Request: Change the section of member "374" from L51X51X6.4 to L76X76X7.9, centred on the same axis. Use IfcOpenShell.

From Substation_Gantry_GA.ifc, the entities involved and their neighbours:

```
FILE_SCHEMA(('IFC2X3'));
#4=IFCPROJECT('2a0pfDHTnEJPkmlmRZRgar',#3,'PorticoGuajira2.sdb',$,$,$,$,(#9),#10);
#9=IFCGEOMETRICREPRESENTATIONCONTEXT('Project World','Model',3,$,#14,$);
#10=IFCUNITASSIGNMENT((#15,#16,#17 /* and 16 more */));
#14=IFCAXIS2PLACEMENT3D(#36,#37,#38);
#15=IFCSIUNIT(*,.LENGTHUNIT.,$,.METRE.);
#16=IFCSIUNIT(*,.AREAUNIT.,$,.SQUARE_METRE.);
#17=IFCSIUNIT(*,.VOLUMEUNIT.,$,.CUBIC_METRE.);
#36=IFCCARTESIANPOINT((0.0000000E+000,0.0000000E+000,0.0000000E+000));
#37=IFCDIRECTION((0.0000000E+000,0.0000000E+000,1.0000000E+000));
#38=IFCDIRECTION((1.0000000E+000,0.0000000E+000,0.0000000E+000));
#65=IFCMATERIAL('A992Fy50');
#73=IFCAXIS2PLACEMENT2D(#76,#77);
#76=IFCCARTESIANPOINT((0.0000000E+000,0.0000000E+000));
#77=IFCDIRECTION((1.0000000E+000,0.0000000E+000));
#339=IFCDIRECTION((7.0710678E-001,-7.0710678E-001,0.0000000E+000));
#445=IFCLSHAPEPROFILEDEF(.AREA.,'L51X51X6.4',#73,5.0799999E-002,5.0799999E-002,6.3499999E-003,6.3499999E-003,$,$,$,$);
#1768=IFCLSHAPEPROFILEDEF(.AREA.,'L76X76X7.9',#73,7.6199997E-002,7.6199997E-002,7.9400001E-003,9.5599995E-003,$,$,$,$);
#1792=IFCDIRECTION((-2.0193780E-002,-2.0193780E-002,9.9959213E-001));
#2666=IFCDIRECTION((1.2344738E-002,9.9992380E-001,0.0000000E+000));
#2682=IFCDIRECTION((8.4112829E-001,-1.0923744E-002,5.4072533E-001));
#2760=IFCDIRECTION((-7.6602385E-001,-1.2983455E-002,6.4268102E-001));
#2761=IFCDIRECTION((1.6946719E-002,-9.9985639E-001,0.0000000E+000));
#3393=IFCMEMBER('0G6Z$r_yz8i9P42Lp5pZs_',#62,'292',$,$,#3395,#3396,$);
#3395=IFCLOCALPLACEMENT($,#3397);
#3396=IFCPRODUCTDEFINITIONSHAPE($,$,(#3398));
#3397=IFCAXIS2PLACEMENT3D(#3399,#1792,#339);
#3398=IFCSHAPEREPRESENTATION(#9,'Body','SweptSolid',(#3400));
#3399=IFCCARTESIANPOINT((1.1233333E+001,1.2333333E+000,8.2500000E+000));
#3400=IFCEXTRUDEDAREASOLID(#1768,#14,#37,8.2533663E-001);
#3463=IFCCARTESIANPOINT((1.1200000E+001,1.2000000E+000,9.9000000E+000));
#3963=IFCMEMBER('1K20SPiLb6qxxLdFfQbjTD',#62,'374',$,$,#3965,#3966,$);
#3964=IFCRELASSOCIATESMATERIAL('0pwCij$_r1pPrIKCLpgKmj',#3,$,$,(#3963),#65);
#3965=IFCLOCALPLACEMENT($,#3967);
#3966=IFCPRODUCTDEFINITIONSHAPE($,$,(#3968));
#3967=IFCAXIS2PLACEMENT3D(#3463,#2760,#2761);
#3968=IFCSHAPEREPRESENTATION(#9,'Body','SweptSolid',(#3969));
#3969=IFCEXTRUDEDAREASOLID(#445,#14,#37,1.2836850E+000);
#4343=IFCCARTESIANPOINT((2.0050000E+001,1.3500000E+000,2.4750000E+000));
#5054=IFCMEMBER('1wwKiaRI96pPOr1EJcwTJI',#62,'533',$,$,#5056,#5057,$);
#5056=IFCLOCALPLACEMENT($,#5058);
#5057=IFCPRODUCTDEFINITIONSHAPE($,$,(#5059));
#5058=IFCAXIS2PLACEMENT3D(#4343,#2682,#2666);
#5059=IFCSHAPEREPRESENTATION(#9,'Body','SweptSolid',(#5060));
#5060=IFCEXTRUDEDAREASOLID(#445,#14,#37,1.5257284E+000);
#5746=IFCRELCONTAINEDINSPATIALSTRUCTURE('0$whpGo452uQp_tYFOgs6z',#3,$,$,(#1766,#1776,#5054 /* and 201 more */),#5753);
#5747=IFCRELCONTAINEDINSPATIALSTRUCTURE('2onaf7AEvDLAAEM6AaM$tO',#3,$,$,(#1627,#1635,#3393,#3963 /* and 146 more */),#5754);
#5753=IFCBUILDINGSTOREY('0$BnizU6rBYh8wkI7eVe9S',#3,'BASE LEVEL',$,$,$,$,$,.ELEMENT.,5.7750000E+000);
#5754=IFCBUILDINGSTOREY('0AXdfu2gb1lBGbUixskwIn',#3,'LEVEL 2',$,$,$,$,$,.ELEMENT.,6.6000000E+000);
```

```python
import ifcopenshell
import ifcopenshell.util.element

model = ifcopenshell.open("Substation_Gantry_GA.ifc")

member = model.by_guid("1K20SPiLb6qxxLdFfQbjTD")
source = next(p for p in model.by_type("IfcLShapeProfileDef") if p.ProfileName == "L76X76X7.9")

body = next(r for r in member.Representation.Representations if r.RepresentationIdentifier == "Body")
solid = body.Items[0]
old_profile = solid.SweptArea

# Copy the section's sizes but keep this member's own profile position.
profile = ifcopenshell.util.element.copy(model, source)
profile.Position = old_profile.Position
solid.SweptArea = profile
if not model.get_total_inverses(old_profile):
    ifcopenshell.util.element.remove_deep2(model, old_profile)

print(solid.SweptArea)

model.write("Substation_Gantry_GA_updated.ifc")
```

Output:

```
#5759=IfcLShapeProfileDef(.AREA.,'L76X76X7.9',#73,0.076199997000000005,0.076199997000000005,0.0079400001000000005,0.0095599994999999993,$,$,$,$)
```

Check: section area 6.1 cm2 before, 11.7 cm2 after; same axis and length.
